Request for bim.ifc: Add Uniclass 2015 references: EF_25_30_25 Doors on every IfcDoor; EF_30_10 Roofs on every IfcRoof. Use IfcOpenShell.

First a look at what the model holds.

```python
import ifcopenshell

model = ifcopenshell.open("bim.ifc")
print(model.schema)
print("classifications:", [c.Name for c in model.by_type("IfcClassification")])
for ifc_class in ("IfcDoor", "IfcRoof", "IfcStair", "IfcWall", "IfcWindow"):
    print(ifc_class, len(model.by_type(ifc_class)))
```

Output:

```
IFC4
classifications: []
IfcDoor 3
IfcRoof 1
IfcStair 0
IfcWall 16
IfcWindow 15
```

```python
import ifcopenshell
import ifcopenshell.api.classification

model = ifcopenshell.open("bim.ifc")

system = ifcopenshell.api.classification.add_classification(model, classification="Uniclass 2015")

codes = {
    "IfcDoor": ("EF_25_30_25", "Doors"),
    "IfcRoof": ("EF_30_10", "Roofs"),
}
for ifc_class, (code, name) in codes.items():
    products = model.by_type(ifc_class)
    ifcopenshell.api.classification.add_reference(
        model, products=products, classification=system, identification=code, name=name
    )
    print(code, len(products))

model.write("bim_v2.ifc")
```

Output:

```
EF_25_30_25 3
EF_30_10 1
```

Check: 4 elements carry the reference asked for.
